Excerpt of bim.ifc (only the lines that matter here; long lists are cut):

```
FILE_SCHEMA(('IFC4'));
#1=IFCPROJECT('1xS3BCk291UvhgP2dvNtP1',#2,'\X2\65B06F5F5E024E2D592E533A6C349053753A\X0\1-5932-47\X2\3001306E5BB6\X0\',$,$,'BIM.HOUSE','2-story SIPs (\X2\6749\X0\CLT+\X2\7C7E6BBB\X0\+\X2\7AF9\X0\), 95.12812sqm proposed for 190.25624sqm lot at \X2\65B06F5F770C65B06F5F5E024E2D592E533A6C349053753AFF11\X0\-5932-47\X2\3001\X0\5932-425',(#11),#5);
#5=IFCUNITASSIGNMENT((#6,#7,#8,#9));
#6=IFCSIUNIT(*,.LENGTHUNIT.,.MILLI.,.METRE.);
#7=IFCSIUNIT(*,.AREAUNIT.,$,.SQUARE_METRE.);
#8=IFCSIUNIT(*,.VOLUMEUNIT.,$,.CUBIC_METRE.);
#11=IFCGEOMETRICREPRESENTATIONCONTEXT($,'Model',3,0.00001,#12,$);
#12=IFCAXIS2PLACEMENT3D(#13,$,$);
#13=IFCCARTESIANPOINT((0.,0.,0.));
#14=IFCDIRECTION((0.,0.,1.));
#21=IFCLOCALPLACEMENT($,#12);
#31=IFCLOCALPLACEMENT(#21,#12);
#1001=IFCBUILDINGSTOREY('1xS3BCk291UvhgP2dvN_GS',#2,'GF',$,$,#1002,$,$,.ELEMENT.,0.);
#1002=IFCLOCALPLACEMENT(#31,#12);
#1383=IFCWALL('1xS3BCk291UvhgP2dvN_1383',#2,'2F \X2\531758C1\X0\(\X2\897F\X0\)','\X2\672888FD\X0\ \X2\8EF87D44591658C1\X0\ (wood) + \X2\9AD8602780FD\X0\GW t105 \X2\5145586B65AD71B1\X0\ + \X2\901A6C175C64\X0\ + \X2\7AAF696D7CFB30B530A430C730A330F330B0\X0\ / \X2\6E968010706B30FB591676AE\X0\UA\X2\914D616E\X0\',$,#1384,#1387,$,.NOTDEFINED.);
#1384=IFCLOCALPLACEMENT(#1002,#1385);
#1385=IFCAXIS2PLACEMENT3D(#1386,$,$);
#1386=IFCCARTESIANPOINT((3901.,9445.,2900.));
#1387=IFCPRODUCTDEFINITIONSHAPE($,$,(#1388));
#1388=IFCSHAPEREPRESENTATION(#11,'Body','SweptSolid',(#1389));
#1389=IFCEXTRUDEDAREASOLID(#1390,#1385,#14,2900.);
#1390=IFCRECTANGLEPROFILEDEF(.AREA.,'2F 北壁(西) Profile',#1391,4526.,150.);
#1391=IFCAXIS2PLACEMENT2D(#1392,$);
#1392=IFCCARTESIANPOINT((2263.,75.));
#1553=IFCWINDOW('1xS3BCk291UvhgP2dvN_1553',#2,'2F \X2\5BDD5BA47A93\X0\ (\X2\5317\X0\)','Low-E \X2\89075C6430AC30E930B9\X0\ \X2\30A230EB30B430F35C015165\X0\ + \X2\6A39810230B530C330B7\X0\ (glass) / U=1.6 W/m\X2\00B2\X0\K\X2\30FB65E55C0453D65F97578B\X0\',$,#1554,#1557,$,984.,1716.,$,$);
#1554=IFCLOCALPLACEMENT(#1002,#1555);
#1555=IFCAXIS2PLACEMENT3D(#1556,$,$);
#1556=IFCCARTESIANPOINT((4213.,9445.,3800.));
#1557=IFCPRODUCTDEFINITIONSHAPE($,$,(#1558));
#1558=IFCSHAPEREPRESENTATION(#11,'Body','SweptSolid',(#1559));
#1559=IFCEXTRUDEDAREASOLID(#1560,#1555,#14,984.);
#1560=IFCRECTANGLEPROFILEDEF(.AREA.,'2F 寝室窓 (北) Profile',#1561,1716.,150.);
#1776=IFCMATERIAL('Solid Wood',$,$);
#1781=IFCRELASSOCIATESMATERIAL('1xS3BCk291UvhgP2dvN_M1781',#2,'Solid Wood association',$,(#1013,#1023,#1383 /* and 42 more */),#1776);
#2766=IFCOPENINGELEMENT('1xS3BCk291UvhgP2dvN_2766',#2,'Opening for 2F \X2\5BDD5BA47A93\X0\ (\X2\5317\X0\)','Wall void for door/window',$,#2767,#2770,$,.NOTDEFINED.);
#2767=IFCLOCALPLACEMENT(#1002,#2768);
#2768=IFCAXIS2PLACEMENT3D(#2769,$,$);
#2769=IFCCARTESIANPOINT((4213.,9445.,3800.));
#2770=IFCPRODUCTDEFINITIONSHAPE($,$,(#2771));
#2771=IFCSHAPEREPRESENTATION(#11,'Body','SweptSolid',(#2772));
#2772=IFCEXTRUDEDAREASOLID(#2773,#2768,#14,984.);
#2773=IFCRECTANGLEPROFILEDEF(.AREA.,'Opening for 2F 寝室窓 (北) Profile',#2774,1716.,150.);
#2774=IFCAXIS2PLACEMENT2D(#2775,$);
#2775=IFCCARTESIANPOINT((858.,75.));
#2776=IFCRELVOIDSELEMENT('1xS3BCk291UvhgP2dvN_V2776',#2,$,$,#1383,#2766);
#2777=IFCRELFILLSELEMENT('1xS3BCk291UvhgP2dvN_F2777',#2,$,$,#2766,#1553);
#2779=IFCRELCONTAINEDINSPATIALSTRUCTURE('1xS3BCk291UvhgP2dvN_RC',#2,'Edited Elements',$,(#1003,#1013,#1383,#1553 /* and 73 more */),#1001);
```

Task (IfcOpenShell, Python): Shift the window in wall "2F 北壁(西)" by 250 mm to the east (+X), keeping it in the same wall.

```python
import ifcopenshell
import ifcopenshell.api.geometry
import ifcopenshell.util.placement

model = ifcopenshell.open("bim.ifc")

window = model.by_id(1553)
opening = window.FillsVoids[0].RelatingOpeningElement
wall = opening.VoidsElements[0].RelatingBuildingElement

wall_matrix = ifcopenshell.util.placement.get_local_placement(wall.ObjectPlacement)
shift = wall_matrix[:3, 0] * 250.0
before = ifcopenshell.util.placement.get_local_placement(window.ObjectPlacement)[:3, 3].copy()

# The window is not placed relative to its opening, so move both.
for product in (opening, window):
    matrix = ifcopenshell.util.placement.get_local_placement(product.ObjectPlacement)
    matrix[:3, 3] += shift
    ifcopenshell.api.geometry.edit_object_placement(model, product=product, matrix=matrix, is_si=False)

after = ifcopenshell.util.placement.get_local_placement(window.ObjectPlacement)[:3, 3]
print("window moved by", (after - before).round(3) + 0.0)

model.write("bim-out.ifc")
```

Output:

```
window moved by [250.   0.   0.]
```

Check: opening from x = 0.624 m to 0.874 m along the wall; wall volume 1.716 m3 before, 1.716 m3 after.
